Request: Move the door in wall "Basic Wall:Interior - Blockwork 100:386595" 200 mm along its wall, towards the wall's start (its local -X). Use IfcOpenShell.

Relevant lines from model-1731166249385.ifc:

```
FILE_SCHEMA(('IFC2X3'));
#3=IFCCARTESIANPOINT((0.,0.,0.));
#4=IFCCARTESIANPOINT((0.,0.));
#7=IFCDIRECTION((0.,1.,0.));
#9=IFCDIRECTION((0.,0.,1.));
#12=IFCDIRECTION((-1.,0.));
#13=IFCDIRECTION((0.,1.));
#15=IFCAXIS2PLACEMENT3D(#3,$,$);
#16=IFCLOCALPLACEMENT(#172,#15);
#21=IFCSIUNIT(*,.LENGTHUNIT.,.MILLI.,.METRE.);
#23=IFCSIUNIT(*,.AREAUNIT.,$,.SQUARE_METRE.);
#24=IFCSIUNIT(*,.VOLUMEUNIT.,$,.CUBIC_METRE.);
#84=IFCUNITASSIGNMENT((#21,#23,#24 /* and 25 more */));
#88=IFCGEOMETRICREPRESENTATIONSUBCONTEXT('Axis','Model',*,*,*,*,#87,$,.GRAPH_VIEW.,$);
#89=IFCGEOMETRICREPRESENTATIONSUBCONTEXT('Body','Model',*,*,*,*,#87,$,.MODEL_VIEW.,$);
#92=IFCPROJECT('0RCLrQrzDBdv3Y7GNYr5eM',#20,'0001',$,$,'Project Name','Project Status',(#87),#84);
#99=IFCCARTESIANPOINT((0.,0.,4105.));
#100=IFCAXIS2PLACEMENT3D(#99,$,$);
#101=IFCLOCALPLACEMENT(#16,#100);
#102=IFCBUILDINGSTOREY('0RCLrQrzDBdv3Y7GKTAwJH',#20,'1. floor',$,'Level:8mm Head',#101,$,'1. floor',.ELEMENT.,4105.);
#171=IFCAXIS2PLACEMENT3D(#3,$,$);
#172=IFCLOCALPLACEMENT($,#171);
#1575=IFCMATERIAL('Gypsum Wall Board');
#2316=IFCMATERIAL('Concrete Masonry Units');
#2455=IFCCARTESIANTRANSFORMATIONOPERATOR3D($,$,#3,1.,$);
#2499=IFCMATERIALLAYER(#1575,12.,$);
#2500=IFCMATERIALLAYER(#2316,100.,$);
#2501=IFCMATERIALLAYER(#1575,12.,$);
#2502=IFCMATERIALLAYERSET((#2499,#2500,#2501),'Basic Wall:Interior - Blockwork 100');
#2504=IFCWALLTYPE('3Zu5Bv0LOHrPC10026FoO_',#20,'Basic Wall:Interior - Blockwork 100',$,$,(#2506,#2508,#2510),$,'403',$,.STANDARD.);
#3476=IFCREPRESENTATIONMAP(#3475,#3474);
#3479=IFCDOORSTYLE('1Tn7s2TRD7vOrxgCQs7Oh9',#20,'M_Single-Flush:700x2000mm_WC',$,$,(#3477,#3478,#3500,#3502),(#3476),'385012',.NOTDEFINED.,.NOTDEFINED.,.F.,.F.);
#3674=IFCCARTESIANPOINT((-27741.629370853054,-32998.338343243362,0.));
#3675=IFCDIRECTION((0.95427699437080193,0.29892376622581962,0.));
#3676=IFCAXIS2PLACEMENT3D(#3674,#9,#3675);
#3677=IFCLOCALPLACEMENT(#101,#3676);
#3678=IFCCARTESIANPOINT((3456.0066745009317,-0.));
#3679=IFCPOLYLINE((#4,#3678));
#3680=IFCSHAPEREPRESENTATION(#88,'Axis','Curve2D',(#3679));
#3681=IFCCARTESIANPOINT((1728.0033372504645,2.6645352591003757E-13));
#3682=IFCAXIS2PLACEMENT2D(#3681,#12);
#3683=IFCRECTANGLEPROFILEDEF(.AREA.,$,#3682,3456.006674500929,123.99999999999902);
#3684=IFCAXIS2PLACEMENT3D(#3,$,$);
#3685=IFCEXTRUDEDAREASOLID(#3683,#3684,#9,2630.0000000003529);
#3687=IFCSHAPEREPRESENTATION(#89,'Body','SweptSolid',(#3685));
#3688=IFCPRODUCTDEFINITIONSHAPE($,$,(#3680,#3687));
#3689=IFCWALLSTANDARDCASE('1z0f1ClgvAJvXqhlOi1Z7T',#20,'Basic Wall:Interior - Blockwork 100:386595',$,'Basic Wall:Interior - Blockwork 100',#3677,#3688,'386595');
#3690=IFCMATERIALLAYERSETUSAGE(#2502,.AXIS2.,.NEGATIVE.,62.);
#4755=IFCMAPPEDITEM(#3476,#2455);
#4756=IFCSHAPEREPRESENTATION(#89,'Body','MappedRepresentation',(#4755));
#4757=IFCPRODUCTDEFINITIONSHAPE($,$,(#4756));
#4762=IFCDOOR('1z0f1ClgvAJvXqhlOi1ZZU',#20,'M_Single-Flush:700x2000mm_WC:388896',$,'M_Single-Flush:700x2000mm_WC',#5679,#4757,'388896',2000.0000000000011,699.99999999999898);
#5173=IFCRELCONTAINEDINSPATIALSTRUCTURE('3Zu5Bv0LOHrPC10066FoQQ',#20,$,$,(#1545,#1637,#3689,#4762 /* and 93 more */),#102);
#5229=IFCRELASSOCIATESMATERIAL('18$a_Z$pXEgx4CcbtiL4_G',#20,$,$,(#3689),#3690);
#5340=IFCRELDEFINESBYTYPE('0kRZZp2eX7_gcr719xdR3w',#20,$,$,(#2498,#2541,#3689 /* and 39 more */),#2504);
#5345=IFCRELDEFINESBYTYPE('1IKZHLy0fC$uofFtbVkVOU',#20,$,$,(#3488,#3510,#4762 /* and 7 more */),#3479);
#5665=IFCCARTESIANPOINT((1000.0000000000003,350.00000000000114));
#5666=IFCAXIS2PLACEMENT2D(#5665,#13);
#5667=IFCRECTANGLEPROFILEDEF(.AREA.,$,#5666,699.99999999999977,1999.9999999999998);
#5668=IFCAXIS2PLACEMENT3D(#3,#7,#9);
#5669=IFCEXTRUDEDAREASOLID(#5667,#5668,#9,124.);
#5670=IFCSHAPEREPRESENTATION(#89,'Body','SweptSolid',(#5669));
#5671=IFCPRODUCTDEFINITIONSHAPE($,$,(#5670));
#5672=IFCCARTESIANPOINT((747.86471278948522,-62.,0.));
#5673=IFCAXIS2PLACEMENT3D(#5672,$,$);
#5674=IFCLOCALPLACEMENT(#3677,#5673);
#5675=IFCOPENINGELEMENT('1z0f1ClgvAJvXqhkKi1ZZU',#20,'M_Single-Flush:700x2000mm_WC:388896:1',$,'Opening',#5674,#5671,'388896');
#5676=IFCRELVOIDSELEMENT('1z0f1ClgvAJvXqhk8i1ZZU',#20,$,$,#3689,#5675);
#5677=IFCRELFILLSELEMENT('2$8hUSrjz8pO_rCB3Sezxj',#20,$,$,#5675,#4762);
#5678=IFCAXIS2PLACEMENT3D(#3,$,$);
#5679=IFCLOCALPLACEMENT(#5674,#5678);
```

```python
import ifcopenshell
import ifcopenshell.api.geometry
import ifcopenshell.util.placement
import ifcopenshell.util.unit

model = ifcopenshell.open("model-1731166249385.ifc")
unit_scale = ifcopenshell.util.unit.calculate_unit_scale(model)

door = model.by_id(4762)
opening = door.FillsVoids[0].RelatingOpeningElement
wall = opening.VoidsElements[0].RelatingBuildingElement

wall_matrix = ifcopenshell.util.placement.get_local_placement(wall.ObjectPlacement)
shift = wall_matrix[:3, 0] * -0.2 / unit_scale
before = ifcopenshell.util.placement.get_local_placement(door.ObjectPlacement)[:3, 3].copy()

# The door is placed relative to its opening, so it follows when the opening moves.
matrix = ifcopenshell.util.placement.get_local_placement(opening.ObjectPlacement)
matrix[:3, 3] += shift
ifcopenshell.api.geometry.edit_object_placement(
    model, product=opening, matrix=matrix, is_si=False, should_transform_children=True
)

after = ifcopenshell.util.placement.get_local_placement(door.ObjectPlacement)[:3, 3]
print("door moved by", (after - before).round(3) + 0.0)

model.write("model-1731166249385_v2.ifc")
```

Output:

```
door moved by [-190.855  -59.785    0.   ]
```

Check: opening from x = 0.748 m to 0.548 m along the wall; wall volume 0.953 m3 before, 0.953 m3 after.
